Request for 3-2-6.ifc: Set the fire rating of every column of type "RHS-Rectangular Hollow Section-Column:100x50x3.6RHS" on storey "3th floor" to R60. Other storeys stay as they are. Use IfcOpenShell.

First a look at what the model holds.

```python
import ifcopenshell
import ifcopenshell.util.element

model = ifcopenshell.open("3-2-6.ifc")
print(model.schema)
storey = next(s for s in model.by_type("IfcBuildingStorey") if s.Name == "3th floor")
columns = [e for e in ifcopenshell.util.element.get_decomposition(storey) if e.is_a("IfcColumn")]
seen = {}
for e in columns:
    element_type = ifcopenshell.util.element.get_type(e)
    key = (element_type.Name if element_type != e and element_type else None, ifcopenshell.util.element.get_pset(e, "Pset_ColumnCommon", "FireRating"))
    seen[key] = seen.get(key, 0) + 1
for (name, value), count in sorted(seen.items(), key=str):
    print(count, "x", name, "|", value)
```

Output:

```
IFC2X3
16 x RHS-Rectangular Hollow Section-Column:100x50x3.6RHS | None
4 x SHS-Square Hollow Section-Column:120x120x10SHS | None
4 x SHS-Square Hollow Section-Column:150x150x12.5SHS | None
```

```python
import ifcopenshell
import ifcopenshell.api.pset
import ifcopenshell.util.element

model = ifcopenshell.open("3-2-6.ifc")

storey = next(s for s in model.by_type("IfcBuildingStorey") if s.Name == "3th floor")
columns = [e for e in ifcopenshell.util.element.get_decomposition(storey) if e.is_a("IfcColumn")]

count = 0
for e in columns:
    element_type = ifcopenshell.util.element.get_type(e)
    if element_type in (None, e) or element_type.Name != "RHS-Rectangular Hollow Section-Column:100x50x3.6RHS":
        continue
    # add_pset returns the element's existing set when there is one.
    pset = ifcopenshell.api.pset.add_pset(model, product=e, name="Pset_ColumnCommon")
    ifcopenshell.api.pset.edit_pset(model, pset=pset, properties={"FireRating": "R60"})
    count += 1

print(count, "columns updated")

model.write("3-2-6_v2.ifc")
```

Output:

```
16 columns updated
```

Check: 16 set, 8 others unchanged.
